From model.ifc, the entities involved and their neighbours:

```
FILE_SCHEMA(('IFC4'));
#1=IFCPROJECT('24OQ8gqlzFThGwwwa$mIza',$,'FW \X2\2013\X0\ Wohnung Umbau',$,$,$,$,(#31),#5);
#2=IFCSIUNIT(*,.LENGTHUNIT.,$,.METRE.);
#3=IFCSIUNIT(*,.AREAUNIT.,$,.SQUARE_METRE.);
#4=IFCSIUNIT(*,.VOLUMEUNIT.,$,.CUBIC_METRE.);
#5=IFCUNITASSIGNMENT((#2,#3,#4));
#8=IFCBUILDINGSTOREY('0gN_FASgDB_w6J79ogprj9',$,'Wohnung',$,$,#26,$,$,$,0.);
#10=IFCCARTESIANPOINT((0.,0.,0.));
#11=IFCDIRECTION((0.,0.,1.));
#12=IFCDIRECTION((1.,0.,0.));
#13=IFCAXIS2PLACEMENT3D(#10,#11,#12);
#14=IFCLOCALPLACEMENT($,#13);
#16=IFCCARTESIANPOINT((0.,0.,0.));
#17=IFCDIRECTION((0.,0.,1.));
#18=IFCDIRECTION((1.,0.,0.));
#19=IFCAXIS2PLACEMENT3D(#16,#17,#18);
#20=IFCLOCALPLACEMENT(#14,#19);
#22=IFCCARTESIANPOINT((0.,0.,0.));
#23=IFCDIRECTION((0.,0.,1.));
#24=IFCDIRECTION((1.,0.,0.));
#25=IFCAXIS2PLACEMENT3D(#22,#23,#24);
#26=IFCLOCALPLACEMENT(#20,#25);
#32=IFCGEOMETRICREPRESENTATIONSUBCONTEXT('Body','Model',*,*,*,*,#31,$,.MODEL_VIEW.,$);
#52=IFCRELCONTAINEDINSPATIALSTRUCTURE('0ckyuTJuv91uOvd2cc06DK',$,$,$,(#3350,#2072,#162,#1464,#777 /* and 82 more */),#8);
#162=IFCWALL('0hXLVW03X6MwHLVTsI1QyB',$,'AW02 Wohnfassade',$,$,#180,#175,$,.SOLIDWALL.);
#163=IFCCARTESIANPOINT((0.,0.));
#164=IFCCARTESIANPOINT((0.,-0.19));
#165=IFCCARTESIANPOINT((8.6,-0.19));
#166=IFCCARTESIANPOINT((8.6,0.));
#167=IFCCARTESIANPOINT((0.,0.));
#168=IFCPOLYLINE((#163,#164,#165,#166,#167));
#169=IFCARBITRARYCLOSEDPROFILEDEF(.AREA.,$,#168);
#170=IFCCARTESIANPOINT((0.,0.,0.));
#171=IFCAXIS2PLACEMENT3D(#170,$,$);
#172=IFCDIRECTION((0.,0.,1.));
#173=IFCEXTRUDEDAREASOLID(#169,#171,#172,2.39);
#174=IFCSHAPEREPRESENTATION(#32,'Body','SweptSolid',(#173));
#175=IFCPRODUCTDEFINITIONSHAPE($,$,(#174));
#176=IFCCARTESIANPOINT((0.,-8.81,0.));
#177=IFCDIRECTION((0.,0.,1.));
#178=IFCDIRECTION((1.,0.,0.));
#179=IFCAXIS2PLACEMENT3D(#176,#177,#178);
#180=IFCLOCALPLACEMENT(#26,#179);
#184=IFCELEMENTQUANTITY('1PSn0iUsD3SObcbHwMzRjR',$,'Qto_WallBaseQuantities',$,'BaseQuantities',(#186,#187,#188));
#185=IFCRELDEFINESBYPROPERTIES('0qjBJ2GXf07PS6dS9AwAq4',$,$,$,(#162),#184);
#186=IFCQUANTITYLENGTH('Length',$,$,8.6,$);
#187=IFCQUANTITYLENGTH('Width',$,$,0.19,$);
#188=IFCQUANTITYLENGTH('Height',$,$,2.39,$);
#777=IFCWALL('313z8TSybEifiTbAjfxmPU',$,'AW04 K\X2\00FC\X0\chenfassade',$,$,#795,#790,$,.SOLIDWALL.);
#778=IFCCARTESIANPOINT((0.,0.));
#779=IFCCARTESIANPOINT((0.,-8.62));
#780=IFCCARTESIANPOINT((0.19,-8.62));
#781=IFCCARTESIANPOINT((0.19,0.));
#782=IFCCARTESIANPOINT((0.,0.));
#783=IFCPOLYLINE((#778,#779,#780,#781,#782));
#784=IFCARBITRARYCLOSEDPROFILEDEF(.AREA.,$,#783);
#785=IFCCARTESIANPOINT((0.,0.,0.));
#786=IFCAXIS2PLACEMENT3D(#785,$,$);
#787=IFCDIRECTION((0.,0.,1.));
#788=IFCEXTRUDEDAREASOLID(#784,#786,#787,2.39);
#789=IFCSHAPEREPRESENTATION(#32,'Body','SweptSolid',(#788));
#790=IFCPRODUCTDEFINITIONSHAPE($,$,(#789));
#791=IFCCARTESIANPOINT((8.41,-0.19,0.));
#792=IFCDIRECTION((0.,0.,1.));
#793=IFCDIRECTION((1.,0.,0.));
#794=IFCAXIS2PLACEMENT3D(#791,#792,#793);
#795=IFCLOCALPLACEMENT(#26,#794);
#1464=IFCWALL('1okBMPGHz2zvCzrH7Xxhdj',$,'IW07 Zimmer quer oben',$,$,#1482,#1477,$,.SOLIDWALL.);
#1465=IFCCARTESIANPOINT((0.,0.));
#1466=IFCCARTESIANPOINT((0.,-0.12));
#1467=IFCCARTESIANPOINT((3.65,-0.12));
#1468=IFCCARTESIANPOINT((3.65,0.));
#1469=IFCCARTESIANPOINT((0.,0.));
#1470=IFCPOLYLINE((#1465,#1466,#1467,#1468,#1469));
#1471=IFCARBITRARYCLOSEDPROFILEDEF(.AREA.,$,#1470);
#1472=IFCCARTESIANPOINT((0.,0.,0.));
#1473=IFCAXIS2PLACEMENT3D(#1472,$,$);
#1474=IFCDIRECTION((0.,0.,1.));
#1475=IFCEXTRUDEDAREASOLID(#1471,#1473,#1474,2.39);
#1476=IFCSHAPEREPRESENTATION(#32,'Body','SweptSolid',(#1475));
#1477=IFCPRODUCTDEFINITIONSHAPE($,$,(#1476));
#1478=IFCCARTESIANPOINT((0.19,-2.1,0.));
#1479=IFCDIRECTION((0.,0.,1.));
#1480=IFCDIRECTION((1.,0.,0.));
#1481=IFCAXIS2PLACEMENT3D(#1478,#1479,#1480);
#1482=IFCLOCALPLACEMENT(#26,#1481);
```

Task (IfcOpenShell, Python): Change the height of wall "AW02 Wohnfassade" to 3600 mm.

```python
import ifcopenshell
import ifcopenshell.api.pset
import ifcopenshell.geom
import ifcopenshell.util.element
import ifcopenshell.util.representation
import ifcopenshell.util.shape
import ifcopenshell.util.unit

model = ifcopenshell.open("model.ifc")
unit_scale = ifcopenshell.util.unit.calculate_unit_scale(model)
settings = ifcopenshell.geom.settings()


def volume(element):
    """Net volume in cubic metres, openings subtracted."""
    shape = ifcopenshell.geom.create_shape(settings, element)
    return ifcopenshell.util.shape.get_volume(shape.geometry)


wall = model.by_guid("0hXLVW03X6MwHLVTsI1QyB")
before = volume(wall)

body = ifcopenshell.util.representation.get_representation(wall, "Model", "Body")
solid = body.Items[0]
old_height = solid.Depth
solid.Depth = 3.6 / unit_scale
after = volume(wall)

# Update the stored height, areas and volumes.
qto = model.by_id(ifcopenshell.util.element.get_pset(wall, "Qto_WallBaseQuantities", should_inherit=False)["id"])
ifcopenshell.api.pset.edit_qto(model, qto=qto, properties={"Height": solid.Depth})

print(f"height {old_height:g} -> {solid.Depth:g}, volume {before:.3f} -> {after:.3f} m3")

model.write("model_v2.ifc")
```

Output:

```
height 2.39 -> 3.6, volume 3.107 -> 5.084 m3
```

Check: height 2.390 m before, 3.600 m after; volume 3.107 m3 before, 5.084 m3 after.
